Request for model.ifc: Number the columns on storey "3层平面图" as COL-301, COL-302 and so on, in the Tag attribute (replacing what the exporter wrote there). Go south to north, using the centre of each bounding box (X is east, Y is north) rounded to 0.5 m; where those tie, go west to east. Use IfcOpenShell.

First a look at what the model holds.

```python
import ifcopenshell
import ifcopenshell.util.element
import ifcopenshell.util.placement

model = ifcopenshell.open("model.ifc")
print(model.schema)
storey = next(s for s in model.by_type("IfcBuildingStorey") if s.Name == "3层平面图")
columns = [e for e in ifcopenshell.util.element.get_decomposition(storey) if e.is_a("IfcColumn")]
for e in sorted(columns, key=lambda e: e.id()):
    origin = ifcopenshell.util.placement.get_local_placement(e.ObjectPlacement)[:3, 3]
    print(e.id(), e.Tag, e.Name, origin.round(2) + 0.0, sep=" | ")
```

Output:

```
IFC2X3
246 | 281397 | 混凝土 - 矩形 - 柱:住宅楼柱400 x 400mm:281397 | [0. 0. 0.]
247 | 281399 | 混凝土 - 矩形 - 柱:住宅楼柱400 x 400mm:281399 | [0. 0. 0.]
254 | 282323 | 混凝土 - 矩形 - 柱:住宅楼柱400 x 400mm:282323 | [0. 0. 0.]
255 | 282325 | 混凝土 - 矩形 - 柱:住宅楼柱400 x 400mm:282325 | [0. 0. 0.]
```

```python
import ifcopenshell
import ifcopenshell.geom
import ifcopenshell.util.element
import ifcopenshell.util.shape

model = ifcopenshell.open("model.ifc")
settings = ifcopenshell.geom.settings()
settings.set("use-world-coords", True)


def centre(element):
    shape = ifcopenshell.geom.create_shape(settings, element)
    return ifcopenshell.util.shape.get_bbox_centroid(shape.geometry)


storey = next(s for s in model.by_type("IfcBuildingStorey") if s.Name == "3层平面图")
columns = [e for e in ifcopenshell.util.element.get_decomposition(storey) if e.is_a("IfcColumn")]

# Insertion points can sit at a corner or the storey origin, so sort by the geometry (in metres).
centres = {e: centre(e) for e in columns}
columns.sort(key=lambda e: (round(centres[e][1] / 0.5), centres[e][0]))

for i, e in enumerate(columns, start=1):
    number = f"COL-3{i:02d}"
    e.Tag = number
    print(e.id(), number)

model.write("model_rev.ifc")
```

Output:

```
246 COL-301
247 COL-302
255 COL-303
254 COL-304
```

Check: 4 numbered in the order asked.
